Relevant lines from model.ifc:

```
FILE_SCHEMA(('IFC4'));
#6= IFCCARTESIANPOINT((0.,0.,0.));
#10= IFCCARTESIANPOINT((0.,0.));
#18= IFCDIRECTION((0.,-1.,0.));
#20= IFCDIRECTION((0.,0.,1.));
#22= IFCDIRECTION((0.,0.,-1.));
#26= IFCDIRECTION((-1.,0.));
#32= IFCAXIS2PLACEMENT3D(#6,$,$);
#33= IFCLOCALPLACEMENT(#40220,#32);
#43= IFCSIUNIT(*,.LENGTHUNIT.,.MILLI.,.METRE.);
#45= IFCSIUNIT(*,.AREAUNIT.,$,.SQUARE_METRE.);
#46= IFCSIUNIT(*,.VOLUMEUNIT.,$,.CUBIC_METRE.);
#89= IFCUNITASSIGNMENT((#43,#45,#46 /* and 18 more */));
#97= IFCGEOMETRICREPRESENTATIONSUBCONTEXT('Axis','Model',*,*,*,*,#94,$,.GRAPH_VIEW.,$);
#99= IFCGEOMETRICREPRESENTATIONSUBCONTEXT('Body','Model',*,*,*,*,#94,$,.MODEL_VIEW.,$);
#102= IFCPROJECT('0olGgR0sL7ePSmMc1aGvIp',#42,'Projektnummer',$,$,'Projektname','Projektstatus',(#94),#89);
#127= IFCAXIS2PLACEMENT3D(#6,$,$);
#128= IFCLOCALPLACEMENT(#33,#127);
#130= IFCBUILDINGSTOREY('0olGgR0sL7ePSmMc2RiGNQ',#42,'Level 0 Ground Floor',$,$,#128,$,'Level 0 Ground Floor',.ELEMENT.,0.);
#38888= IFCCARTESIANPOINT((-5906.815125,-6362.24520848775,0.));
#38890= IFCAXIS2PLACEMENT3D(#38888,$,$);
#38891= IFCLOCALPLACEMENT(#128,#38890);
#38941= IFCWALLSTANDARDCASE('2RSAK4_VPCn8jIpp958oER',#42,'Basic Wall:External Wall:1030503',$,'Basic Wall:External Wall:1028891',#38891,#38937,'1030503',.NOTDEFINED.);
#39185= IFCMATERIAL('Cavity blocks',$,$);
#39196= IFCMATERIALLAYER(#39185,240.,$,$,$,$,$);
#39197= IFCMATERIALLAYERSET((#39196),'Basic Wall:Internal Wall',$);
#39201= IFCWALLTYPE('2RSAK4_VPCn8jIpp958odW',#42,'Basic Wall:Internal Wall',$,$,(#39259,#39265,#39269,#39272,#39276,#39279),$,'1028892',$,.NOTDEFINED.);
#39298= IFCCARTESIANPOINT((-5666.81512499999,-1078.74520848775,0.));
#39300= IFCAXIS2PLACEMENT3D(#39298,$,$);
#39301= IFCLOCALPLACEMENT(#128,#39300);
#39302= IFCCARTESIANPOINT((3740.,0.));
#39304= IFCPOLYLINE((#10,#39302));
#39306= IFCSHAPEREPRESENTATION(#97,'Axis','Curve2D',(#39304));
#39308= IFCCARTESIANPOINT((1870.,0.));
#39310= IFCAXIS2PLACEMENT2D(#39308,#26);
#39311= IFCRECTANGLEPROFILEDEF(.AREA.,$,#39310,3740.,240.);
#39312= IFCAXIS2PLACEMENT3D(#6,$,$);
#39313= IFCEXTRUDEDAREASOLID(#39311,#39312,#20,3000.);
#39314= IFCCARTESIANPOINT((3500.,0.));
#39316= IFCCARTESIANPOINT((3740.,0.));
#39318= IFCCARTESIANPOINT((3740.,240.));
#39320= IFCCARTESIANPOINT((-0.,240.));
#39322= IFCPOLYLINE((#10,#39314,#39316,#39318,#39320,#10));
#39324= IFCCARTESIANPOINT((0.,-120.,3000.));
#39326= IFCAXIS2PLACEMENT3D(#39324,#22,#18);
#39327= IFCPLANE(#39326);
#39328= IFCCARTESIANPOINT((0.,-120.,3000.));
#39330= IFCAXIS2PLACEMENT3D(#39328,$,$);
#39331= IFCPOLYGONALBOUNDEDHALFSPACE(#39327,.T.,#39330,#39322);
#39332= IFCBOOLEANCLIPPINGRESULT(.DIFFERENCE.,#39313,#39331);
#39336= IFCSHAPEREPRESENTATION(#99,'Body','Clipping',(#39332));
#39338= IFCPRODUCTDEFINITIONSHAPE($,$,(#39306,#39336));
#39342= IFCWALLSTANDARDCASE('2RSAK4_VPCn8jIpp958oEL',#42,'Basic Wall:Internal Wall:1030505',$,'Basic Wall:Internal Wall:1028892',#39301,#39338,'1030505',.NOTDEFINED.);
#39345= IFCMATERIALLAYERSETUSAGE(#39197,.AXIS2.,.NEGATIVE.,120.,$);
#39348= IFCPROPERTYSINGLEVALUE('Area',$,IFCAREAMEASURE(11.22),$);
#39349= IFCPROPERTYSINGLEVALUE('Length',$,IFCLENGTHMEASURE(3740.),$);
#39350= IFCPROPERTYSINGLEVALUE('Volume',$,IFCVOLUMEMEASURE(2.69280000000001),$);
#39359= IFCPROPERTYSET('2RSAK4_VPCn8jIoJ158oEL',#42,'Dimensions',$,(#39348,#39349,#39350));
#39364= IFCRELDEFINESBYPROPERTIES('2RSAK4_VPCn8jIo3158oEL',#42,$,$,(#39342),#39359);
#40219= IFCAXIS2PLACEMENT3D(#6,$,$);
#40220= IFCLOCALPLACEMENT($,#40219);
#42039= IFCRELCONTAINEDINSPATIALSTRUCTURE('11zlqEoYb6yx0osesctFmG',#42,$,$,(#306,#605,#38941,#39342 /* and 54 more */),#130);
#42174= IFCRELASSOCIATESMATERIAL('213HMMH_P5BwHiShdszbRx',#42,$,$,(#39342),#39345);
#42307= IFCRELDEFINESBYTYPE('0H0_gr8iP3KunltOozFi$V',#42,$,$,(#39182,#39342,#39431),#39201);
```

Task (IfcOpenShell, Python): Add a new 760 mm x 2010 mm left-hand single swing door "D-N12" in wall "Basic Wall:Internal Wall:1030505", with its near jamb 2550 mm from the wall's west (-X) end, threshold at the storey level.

```python
import numpy as np
import ifcopenshell
import ifcopenshell.api.feature
import ifcopenshell.api.geometry
import ifcopenshell.api.pset
import ifcopenshell.api.root
import ifcopenshell.api.spatial
import ifcopenshell.geom
import ifcopenshell.util.element
import ifcopenshell.util.placement
import ifcopenshell.util.representation
import ifcopenshell.util.shape
import ifcopenshell.util.unit

model = ifcopenshell.open("model.ifc")
unit_scale = ifcopenshell.util.unit.calculate_unit_scale(model)
area_scale = ifcopenshell.util.unit.calculate_unit_scale(model, "AREAUNIT")
volume_scale = ifcopenshell.util.unit.calculate_unit_scale(model, "VOLUMEUNIT")
settings = ifcopenshell.geom.settings()


def volume(element):
    """Net volume in cubic metres, openings subtracted."""
    shape = ifcopenshell.geom.create_shape(settings, element)
    return ifcopenshell.util.shape.get_volume(shape.geometry)


wall = model.by_id(39342)
storey = ifcopenshell.util.element.get_container(wall, ifc_class="IfcBuildingStorey")
context = ifcopenshell.util.representation.get_context(model, "Model", "Body", "MODEL_VIEW")
before = volume(wall)

width, height, from_end, sill = 0.76, 2.01, 2.55, 0.0  # metres

# The wall runs along its own X axis, and the end named is its -X end.
wall_shape = ifcopenshell.geom.create_shape(settings, wall)
x, y, z = ifcopenshell.util.shape.get_vertices(wall_shape.geometry).T
start = x.min() + from_end
face, thickness = float(y.min()), float(y.max() - y.min())
wall_matrix = ifcopenshell.util.placement.get_local_placement(wall.ObjectPlacement)
level = ifcopenshell.util.placement.get_local_placement(storey.ObjectPlacement)[2, 3]


def in_wall(x, y):
    """Placement at x, y metres in the wall's axes, at sill height."""
    matrix = wall_matrix.copy()
    matrix[:, 3] = wall_matrix @ np.array([x / unit_scale, y / unit_scale, 0.0, 1.0])
    matrix[2, 3] = level + sill / unit_scale
    return matrix


# Opening: a box that overshoots both wall faces by 50 mm.
opening = ifcopenshell.api.root.create_entity(model, ifc_class="IfcOpeningElement", predefined_type="OPENING")
box = ifcopenshell.api.geometry.add_wall_representation(
    model, context=context, length=width, height=height, thickness=thickness + 0.1
)
ifcopenshell.api.geometry.assign_representation(model, product=opening, representation=box)
ifcopenshell.api.geometry.edit_object_placement(model, product=opening, matrix=in_wall(start, face - 0.05), is_si=False)
ifcopenshell.api.feature.add_feature(model, feature=opening, element=wall)

door = ifcopenshell.api.root.create_entity(model, ifc_class="IfcDoor", name="D-N12", predefined_type="DOOR")
door.OverallWidth, door.OverallHeight = width / unit_scale, height / unit_scale
door.OperationType = "SINGLE_SWING_LEFT"
body = ifcopenshell.api.geometry.add_door_representation(
    model,
    context=context,
    overall_width=door.OverallWidth,
    overall_height=door.OverallHeight,
    operation_type="SINGLE_SWING_LEFT",
    lining_properties={"LiningDepth": thickness / unit_scale, "ThresholdDepth": thickness / unit_scale},
)
ifcopenshell.api.geometry.assign_representation(model, product=door, representation=body)
ifcopenshell.api.spatial.assign_container(model, products=[door], relating_structure=storey)
ifcopenshell.api.feature.add_filling(model, opening=opening, element=door)

# The lining spans the wall, so the door starts at the wall face.
ifcopenshell.api.geometry.edit_object_placement(model, product=door, matrix=in_wall(start, face), is_si=False)

after = volume(wall)

# Update the wall's stored quantities.
pset = model.by_id(ifcopenshell.util.element.get_pset(wall, "Dimensions", should_inherit=False)["id"])
ifcopenshell.api.pset.edit_pset(model, pset=pset, properties={
    "Area": model.create_entity("IfcAreaMeasure", after / thickness / area_scale),
    "Volume": model.create_entity("IfcVolumeMeasure", after / volume_scale),
})

print(f"wall volume {before:.3f} -> {after:.3f} m3")

model.write("model_edited.ifc")
```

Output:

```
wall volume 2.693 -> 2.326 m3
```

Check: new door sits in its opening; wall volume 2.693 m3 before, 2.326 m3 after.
